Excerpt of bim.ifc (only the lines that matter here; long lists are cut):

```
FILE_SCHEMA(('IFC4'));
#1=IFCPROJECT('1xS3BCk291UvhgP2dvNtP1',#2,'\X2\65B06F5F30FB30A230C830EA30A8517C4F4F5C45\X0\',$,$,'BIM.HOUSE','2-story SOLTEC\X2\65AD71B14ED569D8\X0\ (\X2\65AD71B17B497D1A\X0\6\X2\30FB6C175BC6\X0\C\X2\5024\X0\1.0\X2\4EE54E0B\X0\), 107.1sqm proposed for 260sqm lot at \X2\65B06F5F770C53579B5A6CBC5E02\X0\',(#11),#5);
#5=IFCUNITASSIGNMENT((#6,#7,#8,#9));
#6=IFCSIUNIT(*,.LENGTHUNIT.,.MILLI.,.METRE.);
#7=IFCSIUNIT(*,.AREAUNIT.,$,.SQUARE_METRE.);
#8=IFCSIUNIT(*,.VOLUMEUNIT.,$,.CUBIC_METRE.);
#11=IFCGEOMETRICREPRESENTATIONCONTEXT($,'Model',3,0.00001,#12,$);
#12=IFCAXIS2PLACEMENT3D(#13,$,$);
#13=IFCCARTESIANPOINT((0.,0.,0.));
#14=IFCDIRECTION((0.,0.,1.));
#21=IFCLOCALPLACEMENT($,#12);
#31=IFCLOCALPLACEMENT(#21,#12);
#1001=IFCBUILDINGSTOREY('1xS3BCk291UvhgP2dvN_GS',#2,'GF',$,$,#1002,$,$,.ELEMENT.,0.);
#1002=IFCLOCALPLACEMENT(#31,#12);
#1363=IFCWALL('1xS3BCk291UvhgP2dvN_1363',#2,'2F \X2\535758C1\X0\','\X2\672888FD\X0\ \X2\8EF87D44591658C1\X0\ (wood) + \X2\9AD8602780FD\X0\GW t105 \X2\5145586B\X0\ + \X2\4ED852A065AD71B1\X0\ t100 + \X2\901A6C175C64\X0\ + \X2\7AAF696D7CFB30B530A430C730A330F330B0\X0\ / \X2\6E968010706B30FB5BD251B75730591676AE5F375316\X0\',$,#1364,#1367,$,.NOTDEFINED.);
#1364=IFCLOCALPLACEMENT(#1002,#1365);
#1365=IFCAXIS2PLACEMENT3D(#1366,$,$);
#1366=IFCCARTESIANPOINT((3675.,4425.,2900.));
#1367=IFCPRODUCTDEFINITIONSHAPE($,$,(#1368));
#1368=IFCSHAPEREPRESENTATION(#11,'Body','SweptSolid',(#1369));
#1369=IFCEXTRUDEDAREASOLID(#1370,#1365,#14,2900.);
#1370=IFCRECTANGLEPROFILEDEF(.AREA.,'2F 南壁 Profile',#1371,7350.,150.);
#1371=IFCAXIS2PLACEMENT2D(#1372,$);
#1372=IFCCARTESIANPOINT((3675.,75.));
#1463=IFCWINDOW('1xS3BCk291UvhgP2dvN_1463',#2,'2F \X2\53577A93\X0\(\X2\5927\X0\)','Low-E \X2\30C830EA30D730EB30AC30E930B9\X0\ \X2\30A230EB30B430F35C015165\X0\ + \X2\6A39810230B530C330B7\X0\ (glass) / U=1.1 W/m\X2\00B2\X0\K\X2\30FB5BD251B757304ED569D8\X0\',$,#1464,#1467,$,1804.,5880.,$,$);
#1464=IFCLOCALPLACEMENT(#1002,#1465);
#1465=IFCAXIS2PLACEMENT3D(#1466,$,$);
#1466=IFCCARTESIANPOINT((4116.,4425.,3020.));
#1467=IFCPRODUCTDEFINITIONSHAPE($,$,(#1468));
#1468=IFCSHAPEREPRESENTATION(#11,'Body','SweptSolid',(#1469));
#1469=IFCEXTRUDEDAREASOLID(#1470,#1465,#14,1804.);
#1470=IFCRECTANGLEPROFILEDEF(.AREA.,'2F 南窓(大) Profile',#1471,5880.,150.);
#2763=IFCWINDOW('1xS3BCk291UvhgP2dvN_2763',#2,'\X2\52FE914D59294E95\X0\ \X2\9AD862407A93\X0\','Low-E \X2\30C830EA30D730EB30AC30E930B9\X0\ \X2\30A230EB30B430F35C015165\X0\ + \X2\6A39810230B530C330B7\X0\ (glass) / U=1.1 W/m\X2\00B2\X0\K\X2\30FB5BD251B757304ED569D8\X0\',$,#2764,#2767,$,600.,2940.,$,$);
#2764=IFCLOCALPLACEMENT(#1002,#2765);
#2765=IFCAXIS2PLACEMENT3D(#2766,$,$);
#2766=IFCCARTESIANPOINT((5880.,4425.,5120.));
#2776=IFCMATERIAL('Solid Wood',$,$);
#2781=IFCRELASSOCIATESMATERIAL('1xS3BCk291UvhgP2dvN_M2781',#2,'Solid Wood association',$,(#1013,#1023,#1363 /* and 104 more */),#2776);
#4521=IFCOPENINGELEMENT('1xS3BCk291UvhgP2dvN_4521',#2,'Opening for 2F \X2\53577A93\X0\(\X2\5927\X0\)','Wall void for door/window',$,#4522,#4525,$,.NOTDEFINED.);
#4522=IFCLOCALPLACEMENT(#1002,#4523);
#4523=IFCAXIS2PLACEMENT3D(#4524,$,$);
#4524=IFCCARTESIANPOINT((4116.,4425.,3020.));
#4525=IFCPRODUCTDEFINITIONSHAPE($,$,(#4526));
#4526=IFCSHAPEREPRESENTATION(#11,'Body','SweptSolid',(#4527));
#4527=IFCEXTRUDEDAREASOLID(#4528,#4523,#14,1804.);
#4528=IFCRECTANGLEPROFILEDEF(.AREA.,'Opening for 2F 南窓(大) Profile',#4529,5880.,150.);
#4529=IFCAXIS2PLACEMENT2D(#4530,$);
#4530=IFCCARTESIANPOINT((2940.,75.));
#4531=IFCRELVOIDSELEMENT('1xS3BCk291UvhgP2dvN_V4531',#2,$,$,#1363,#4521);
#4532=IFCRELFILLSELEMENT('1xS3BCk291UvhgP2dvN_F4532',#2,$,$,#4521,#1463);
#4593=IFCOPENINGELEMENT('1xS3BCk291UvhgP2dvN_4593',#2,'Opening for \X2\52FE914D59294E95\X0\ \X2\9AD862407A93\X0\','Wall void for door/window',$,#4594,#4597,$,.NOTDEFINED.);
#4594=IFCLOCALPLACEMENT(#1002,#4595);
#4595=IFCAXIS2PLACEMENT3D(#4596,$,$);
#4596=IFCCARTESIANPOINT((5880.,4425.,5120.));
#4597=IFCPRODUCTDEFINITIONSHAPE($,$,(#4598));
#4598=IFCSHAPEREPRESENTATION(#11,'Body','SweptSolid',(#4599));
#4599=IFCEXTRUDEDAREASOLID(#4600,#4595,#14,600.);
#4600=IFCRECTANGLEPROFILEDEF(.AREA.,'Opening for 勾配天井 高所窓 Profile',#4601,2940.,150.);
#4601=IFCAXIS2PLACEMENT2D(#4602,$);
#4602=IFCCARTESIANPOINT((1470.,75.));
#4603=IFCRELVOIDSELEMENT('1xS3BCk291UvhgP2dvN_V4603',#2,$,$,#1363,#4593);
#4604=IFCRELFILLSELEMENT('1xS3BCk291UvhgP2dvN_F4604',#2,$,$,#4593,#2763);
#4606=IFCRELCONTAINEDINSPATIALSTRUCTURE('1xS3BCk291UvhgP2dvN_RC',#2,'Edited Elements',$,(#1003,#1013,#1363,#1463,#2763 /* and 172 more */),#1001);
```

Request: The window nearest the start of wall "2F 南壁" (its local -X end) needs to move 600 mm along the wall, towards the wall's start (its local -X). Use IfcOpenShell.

```python
import ifcopenshell
import ifcopenshell.api.geometry
import ifcopenshell.util.placement
import ifcopenshell.util.unit

model = ifcopenshell.open("bim.ifc")
unit_scale = ifcopenshell.util.unit.calculate_unit_scale(model)

window = model.by_guid("1xS3BCk291UvhgP2dvN_1463")
opening = window.FillsVoids[0].RelatingOpeningElement
wall = opening.VoidsElements[0].RelatingBuildingElement

wall_matrix = ifcopenshell.util.placement.get_local_placement(wall.ObjectPlacement)
shift = wall_matrix[:3, 0] * -0.6 / unit_scale
before = ifcopenshell.util.placement.get_local_placement(window.ObjectPlacement)[:3, 3].copy()

# The window is not placed relative to its opening, so move both.
for product in (opening, window):
    matrix = ifcopenshell.util.placement.get_local_placement(product.ObjectPlacement)
    matrix[:3, 3] += shift
    ifcopenshell.api.geometry.edit_object_placement(model, product=product, matrix=matrix, is_si=False)

after = ifcopenshell.util.placement.get_local_placement(window.ObjectPlacement)[:3, 3]
print("window moved by", (after - before).round(3) + 0.0)

model.write("bim_v2.ifc")
```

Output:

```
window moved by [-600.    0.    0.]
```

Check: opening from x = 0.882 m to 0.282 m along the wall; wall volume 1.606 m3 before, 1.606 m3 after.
